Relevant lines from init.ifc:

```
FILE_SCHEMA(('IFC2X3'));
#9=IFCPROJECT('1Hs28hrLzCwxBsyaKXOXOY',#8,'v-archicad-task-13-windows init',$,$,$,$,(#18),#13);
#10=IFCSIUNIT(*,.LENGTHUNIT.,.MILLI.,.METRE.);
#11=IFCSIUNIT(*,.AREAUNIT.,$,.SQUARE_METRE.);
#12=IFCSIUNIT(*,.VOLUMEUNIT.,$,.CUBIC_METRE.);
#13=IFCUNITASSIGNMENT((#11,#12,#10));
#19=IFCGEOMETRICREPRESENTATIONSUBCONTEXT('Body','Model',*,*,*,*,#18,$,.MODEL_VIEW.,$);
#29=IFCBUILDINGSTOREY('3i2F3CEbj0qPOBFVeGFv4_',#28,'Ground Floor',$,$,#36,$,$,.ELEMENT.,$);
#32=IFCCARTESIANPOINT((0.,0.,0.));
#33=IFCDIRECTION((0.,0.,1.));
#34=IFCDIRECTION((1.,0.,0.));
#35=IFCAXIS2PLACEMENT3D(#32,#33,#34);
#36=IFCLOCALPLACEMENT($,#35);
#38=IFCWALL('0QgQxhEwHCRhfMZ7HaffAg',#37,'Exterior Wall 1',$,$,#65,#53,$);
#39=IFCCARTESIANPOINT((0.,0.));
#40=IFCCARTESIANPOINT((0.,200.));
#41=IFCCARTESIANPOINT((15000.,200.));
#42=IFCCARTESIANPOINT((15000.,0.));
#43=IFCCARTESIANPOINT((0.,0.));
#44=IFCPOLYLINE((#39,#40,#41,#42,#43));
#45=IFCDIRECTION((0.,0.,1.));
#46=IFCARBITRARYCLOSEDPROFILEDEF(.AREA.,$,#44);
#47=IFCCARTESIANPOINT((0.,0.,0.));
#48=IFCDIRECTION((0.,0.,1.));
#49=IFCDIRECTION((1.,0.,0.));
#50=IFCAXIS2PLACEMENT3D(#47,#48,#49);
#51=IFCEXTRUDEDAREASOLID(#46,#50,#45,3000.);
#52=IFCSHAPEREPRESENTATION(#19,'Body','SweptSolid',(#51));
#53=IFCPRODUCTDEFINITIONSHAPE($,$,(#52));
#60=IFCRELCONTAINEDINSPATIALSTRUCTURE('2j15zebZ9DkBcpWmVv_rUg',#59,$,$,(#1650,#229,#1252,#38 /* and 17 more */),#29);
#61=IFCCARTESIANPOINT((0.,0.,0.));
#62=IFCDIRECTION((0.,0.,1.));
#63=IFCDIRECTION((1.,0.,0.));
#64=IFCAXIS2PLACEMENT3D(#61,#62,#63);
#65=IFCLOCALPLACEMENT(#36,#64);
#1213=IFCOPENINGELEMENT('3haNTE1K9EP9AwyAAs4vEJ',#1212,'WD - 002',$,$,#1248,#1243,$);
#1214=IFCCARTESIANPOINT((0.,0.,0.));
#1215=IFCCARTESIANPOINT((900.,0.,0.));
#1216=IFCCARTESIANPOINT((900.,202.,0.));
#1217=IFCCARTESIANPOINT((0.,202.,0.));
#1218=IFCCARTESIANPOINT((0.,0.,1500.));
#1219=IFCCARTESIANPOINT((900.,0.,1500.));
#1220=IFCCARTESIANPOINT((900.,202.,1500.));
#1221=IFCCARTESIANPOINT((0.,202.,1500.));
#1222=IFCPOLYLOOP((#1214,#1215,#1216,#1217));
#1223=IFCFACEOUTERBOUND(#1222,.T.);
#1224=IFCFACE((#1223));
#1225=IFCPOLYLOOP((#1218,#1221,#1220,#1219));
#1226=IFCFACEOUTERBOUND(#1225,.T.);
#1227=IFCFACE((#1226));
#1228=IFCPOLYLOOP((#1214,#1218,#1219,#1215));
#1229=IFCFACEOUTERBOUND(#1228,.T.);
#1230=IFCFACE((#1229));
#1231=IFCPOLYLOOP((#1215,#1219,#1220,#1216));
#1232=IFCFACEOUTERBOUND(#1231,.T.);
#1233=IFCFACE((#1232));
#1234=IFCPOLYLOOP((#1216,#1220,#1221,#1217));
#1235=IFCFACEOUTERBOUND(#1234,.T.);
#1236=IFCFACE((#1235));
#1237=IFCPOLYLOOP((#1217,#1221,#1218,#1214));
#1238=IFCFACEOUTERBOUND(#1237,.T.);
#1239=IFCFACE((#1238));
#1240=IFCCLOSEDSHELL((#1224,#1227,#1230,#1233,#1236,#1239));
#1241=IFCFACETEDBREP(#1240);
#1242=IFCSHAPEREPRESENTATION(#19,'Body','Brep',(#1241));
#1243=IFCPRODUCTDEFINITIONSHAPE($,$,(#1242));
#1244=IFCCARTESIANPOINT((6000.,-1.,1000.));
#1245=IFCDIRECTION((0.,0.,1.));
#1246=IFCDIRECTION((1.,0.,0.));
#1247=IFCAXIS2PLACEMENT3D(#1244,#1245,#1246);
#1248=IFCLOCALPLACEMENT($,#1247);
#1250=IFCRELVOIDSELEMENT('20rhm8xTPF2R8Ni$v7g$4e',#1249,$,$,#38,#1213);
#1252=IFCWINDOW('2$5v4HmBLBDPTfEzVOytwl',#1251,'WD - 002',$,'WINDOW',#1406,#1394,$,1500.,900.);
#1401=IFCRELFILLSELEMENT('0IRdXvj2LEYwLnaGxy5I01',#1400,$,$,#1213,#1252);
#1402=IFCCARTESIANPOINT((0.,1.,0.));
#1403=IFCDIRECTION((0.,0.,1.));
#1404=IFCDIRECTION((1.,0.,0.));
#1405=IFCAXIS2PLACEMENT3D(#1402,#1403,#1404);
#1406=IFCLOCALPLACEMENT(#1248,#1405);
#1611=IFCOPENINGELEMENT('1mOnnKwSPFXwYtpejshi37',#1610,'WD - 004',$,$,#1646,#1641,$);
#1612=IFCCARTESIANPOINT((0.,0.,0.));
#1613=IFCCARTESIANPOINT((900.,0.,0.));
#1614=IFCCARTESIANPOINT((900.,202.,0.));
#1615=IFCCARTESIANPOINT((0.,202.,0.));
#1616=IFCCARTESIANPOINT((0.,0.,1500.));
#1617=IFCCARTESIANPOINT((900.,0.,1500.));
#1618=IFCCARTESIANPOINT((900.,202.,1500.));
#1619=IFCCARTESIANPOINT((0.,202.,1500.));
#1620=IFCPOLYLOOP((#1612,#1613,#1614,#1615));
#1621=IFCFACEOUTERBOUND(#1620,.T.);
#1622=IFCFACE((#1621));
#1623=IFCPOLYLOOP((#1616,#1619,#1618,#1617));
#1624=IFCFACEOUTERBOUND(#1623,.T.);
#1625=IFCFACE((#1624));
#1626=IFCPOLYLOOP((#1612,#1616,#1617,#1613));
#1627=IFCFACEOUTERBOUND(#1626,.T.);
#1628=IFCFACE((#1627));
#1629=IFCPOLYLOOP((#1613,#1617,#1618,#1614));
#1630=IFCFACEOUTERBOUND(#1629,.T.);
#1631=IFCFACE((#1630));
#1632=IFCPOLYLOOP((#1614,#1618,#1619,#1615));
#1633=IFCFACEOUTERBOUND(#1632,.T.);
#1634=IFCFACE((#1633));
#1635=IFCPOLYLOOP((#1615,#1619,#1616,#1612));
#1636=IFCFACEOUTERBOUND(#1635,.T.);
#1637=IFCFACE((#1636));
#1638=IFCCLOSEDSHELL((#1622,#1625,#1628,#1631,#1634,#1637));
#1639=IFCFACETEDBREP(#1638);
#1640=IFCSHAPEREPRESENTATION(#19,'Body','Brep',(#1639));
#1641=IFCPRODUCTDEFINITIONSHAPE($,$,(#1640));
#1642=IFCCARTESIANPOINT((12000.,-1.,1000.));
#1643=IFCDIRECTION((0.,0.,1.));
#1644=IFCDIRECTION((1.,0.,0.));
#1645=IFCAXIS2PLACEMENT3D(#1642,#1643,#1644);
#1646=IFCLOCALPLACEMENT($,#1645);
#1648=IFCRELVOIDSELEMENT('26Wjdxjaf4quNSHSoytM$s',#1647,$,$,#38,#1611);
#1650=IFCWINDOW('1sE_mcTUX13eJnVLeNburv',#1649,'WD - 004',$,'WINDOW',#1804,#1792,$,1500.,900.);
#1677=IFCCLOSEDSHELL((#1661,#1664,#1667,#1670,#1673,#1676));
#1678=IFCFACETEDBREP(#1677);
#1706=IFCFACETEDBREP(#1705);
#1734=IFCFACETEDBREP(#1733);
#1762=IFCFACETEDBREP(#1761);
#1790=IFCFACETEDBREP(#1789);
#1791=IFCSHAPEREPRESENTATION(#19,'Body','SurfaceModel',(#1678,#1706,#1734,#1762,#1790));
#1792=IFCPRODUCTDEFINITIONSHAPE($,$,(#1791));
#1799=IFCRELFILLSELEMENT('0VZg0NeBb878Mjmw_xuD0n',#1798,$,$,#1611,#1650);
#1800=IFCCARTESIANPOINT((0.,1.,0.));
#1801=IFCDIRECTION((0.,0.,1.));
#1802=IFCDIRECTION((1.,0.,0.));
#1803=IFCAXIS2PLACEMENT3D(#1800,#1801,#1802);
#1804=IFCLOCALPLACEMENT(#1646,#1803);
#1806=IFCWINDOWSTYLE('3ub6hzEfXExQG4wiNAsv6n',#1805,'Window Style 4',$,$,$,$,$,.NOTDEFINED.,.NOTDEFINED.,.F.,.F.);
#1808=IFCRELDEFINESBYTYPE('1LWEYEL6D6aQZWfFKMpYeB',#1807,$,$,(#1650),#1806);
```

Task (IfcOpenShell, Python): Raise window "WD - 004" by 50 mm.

```python
import numpy as np
import ifcopenshell
import ifcopenshell.api.geometry
import ifcopenshell.util.placement
import ifcopenshell.util.unit

model = ifcopenshell.open("init.ifc")
unit_scale = ifcopenshell.util.unit.calculate_unit_scale(model)

window = model.by_id(1650)
opening = window.FillsVoids[0].RelatingOpeningElement
dz = 50.0

shift = np.array([0.0, 0.0, dz])
# The window is placed relative to its opening, so it follows when the opening moves.
matrix = ifcopenshell.util.placement.get_local_placement(opening.ObjectPlacement)
matrix[:3, 3] += shift
ifcopenshell.api.geometry.edit_object_placement(
    model, product=opening, matrix=matrix, is_si=False, should_transform_children=True
)

print(f"moved by {dz * unit_scale:+.3f} m")

model.write("init_rev.ifc")
```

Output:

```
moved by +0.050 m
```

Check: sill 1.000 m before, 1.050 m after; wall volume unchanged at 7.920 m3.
